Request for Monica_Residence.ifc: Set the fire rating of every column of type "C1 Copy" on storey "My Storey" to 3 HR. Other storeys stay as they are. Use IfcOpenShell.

First a look at what the model holds.

```python
import ifcopenshell
import ifcopenshell.util.element

model = ifcopenshell.open("Monica_Residence.ifc")
print(model.schema)
storey = next(s for s in model.by_type("IfcBuildingStorey") if s.Name == "My Storey")
columns = [e for e in ifcopenshell.util.element.get_decomposition(storey) if e.is_a("IfcColumn")]
seen = {}
for e in columns:
    element_type = ifcopenshell.util.element.get_type(e)
    key = (element_type.Name if element_type != e and element_type else None, ifcopenshell.util.element.get_pset(e, "Pset_ColumnCommon", "FireRating"))
    seen[key] = seen.get(key, 0) + 1
for (name, value), count in sorted(seen.items(), key=str):
    print(count, "x", name, "|", value)
```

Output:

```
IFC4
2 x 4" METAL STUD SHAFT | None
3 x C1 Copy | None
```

```python
import ifcopenshell
import ifcopenshell.api.pset
import ifcopenshell.util.element

model = ifcopenshell.open("Monica_Residence.ifc")

storey = next(s for s in model.by_type("IfcBuildingStorey") if s.Name == "My Storey")
columns = [e for e in ifcopenshell.util.element.get_decomposition(storey) if e.is_a("IfcColumn")]

count = 0
for e in columns:
    element_type = ifcopenshell.util.element.get_type(e)
    if element_type in (None, e) or element_type.Name != "C1 Copy":
        continue
    # add_pset returns the element's existing set when there is one.
    pset = ifcopenshell.api.pset.add_pset(model, product=e, name="Pset_ColumnCommon")
    ifcopenshell.api.pset.edit_pset(model, pset=pset, properties={"FireRating": "3 HR"})
    count += 1

print(count, "columns updated")

model.write("Monica_Residence_updated.ifc")
```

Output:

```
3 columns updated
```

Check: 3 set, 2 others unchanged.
